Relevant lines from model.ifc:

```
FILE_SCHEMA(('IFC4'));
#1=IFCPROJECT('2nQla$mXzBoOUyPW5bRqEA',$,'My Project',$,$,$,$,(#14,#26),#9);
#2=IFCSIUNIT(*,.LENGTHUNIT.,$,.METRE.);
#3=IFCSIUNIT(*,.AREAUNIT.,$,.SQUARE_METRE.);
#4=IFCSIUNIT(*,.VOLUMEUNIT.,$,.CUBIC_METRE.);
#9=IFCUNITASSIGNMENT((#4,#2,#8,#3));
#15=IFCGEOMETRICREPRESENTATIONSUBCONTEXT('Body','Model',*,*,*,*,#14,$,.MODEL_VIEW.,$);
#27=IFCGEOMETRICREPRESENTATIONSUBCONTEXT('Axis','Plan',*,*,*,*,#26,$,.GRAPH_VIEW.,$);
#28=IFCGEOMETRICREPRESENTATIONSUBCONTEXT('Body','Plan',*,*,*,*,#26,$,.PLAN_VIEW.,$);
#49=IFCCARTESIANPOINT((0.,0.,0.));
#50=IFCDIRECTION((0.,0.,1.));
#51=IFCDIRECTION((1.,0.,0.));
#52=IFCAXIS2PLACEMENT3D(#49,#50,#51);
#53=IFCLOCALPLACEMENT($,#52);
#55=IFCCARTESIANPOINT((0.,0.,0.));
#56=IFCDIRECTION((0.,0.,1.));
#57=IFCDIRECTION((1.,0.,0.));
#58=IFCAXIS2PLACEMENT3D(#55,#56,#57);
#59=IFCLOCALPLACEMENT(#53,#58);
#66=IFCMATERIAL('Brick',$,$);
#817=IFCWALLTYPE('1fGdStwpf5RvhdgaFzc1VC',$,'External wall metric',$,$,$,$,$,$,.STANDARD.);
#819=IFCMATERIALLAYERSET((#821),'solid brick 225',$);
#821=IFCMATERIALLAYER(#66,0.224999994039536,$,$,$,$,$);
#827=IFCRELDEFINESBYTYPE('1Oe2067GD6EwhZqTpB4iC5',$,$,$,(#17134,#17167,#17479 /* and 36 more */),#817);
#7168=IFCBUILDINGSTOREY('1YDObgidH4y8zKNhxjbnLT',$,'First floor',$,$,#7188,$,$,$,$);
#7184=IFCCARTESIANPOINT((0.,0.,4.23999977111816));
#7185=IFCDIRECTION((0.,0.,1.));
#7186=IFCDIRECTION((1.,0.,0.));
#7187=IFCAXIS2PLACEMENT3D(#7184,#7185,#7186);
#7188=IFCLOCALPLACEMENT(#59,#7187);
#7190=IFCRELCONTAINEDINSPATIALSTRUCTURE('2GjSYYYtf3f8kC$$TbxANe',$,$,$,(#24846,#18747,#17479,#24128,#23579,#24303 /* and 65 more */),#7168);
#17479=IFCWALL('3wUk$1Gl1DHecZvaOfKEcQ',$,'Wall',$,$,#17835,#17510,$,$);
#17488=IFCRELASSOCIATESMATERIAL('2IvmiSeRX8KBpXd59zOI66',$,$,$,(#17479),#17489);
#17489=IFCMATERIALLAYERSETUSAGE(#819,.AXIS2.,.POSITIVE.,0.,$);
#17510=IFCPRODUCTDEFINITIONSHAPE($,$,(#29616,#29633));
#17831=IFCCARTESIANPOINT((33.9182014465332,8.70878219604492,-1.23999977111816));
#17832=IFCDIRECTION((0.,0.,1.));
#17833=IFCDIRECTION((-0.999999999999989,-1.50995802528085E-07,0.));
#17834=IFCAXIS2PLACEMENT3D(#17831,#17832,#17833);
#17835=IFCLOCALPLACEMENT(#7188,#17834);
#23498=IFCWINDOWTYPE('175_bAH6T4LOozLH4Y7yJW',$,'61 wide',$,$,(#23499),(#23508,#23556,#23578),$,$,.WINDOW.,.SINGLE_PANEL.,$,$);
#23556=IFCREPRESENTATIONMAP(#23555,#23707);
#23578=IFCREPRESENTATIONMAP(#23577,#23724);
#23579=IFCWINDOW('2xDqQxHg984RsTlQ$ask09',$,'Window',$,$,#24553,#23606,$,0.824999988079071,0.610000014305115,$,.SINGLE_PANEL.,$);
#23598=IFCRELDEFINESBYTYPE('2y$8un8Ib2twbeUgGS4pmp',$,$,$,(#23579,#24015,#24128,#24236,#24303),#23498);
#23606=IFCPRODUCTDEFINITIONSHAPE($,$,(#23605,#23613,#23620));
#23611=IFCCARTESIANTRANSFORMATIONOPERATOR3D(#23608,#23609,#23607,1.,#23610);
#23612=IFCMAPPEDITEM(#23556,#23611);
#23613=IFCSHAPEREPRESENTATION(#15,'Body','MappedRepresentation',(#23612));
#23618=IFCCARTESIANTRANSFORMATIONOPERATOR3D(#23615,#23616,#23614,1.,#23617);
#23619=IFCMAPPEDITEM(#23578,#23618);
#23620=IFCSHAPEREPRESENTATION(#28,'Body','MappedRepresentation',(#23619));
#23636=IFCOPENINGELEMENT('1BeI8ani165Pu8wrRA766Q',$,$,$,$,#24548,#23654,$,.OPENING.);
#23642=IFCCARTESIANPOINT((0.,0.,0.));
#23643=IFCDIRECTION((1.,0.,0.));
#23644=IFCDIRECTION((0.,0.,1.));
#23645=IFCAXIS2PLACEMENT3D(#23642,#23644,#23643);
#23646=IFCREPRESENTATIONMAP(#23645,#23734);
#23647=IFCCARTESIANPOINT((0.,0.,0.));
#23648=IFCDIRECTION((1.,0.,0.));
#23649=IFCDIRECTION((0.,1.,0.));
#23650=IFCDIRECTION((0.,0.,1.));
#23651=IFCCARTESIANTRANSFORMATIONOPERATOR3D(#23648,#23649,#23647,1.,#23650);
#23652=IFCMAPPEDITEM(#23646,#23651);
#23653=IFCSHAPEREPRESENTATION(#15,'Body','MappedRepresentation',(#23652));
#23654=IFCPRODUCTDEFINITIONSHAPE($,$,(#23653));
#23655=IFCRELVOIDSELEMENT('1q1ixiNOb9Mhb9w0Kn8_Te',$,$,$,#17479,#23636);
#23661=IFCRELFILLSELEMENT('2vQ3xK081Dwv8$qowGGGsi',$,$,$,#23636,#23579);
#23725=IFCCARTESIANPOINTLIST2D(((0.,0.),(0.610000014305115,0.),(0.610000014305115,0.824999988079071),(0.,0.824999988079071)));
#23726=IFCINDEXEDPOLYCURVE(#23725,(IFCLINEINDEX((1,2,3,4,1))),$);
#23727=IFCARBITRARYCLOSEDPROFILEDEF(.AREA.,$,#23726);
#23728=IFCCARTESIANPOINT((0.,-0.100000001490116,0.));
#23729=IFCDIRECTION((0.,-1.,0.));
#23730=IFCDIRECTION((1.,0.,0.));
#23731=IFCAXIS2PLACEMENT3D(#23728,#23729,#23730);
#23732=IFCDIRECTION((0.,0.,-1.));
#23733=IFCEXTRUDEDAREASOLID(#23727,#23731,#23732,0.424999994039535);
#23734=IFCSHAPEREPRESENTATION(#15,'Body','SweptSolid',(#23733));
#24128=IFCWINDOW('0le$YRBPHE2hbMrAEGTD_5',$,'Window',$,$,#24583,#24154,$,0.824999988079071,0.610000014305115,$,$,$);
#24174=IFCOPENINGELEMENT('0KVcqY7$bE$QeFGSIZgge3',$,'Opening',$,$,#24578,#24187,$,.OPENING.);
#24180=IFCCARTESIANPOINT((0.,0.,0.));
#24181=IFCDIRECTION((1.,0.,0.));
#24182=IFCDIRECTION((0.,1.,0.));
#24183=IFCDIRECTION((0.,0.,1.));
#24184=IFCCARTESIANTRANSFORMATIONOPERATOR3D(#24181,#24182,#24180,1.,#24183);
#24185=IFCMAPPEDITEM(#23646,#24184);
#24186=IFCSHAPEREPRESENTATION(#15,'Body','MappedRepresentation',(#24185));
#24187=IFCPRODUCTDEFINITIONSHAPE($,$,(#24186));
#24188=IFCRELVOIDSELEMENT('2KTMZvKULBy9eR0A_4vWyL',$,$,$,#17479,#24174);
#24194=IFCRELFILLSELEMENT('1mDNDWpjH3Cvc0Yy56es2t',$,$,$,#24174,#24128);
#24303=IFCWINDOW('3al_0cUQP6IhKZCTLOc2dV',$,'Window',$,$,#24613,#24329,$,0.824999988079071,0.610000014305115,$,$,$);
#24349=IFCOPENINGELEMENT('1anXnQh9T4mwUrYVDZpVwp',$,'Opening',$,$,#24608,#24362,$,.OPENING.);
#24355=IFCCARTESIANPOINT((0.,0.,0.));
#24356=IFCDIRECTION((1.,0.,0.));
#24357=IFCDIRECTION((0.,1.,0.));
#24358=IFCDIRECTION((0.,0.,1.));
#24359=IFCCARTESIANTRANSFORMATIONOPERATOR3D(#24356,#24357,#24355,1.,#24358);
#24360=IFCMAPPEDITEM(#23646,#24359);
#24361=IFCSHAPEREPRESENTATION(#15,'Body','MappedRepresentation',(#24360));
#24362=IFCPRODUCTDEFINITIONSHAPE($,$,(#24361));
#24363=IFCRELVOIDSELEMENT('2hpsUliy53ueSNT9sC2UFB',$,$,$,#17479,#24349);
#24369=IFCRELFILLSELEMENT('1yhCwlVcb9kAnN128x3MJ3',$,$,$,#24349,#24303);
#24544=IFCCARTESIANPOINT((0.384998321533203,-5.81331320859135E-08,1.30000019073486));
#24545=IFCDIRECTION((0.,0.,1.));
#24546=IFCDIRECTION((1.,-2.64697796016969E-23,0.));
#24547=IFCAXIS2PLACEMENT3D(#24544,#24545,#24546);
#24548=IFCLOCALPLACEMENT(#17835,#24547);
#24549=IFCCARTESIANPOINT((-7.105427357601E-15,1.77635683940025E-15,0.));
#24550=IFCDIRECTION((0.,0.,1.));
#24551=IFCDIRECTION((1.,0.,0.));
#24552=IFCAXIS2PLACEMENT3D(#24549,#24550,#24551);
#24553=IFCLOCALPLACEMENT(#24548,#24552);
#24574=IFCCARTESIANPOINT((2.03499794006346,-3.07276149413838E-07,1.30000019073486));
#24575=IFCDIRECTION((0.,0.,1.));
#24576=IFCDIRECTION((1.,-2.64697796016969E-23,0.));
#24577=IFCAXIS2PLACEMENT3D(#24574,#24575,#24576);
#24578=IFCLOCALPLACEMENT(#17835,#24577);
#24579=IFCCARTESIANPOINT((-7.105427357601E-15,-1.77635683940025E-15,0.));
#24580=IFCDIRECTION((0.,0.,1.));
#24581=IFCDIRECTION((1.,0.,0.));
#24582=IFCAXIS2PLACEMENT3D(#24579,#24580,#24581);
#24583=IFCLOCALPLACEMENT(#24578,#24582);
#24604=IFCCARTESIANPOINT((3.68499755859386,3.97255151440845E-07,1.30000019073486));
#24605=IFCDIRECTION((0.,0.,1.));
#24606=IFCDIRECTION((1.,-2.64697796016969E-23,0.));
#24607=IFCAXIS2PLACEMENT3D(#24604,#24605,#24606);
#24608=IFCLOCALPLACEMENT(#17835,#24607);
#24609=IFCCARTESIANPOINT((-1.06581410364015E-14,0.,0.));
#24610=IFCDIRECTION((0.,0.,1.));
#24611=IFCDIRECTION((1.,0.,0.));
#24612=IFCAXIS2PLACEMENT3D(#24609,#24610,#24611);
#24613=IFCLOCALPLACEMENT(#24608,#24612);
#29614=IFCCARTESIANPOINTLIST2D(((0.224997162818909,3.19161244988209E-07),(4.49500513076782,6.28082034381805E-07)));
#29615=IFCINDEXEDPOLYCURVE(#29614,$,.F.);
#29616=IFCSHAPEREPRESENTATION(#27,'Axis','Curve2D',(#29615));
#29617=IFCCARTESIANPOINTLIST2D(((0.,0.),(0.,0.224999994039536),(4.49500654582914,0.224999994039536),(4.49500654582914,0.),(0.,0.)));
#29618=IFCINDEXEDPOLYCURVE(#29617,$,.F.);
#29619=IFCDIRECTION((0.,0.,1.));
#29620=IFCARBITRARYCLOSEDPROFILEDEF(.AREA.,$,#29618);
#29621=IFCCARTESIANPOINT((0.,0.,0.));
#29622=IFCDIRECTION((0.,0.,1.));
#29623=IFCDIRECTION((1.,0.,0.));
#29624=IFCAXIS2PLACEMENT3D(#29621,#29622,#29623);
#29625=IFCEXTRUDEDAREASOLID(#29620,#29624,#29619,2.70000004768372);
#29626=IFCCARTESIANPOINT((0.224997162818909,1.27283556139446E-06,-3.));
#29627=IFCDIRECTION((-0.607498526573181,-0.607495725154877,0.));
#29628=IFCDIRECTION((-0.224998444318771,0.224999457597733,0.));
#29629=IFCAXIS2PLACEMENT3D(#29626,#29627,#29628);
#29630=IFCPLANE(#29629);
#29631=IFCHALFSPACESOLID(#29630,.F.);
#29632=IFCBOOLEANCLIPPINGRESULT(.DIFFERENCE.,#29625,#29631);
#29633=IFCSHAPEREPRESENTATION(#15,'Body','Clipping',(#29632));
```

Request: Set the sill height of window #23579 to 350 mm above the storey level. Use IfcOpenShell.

```python
import numpy as np
import ifcopenshell
import ifcopenshell.api.geometry
import ifcopenshell.geom
import ifcopenshell.util.element
import ifcopenshell.util.placement
import ifcopenshell.util.shape
import ifcopenshell.util.unit

model = ifcopenshell.open("model.ifc")
unit_scale = ifcopenshell.util.unit.calculate_unit_scale(model)

window = model.by_id(23579)
opening = window.FillsVoids[0].RelatingOpeningElement
storey = ifcopenshell.util.element.get_container(window, ifc_class="IfcBuildingStorey")
level = ifcopenshell.util.placement.get_local_placement(storey.ObjectPlacement)[2, 3]

# The opening's origin need not be at the sill, so measure its lowest point.
shape = ifcopenshell.geom.create_shape(ifcopenshell.geom.settings(), opening)
bottom = ifcopenshell.util.shape.get_shape_bottom_elevation(shape, shape.geometry) / unit_scale
dz = level + 0.35 - bottom

shift = np.array([0.0, 0.0, dz])
# The window is placed relative to its opening, so it follows when the opening moves.
matrix = ifcopenshell.util.placement.get_local_placement(opening.ObjectPlacement)
matrix[:3, 3] += shift
ifcopenshell.api.geometry.edit_object_placement(
    model, product=opening, matrix=matrix, is_si=False, should_transform_children=True
)

print(f"moved by {dz * unit_scale:+.3f} m")

model.write("model_updated.ifc")
```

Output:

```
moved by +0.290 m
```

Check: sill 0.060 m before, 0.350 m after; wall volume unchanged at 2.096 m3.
